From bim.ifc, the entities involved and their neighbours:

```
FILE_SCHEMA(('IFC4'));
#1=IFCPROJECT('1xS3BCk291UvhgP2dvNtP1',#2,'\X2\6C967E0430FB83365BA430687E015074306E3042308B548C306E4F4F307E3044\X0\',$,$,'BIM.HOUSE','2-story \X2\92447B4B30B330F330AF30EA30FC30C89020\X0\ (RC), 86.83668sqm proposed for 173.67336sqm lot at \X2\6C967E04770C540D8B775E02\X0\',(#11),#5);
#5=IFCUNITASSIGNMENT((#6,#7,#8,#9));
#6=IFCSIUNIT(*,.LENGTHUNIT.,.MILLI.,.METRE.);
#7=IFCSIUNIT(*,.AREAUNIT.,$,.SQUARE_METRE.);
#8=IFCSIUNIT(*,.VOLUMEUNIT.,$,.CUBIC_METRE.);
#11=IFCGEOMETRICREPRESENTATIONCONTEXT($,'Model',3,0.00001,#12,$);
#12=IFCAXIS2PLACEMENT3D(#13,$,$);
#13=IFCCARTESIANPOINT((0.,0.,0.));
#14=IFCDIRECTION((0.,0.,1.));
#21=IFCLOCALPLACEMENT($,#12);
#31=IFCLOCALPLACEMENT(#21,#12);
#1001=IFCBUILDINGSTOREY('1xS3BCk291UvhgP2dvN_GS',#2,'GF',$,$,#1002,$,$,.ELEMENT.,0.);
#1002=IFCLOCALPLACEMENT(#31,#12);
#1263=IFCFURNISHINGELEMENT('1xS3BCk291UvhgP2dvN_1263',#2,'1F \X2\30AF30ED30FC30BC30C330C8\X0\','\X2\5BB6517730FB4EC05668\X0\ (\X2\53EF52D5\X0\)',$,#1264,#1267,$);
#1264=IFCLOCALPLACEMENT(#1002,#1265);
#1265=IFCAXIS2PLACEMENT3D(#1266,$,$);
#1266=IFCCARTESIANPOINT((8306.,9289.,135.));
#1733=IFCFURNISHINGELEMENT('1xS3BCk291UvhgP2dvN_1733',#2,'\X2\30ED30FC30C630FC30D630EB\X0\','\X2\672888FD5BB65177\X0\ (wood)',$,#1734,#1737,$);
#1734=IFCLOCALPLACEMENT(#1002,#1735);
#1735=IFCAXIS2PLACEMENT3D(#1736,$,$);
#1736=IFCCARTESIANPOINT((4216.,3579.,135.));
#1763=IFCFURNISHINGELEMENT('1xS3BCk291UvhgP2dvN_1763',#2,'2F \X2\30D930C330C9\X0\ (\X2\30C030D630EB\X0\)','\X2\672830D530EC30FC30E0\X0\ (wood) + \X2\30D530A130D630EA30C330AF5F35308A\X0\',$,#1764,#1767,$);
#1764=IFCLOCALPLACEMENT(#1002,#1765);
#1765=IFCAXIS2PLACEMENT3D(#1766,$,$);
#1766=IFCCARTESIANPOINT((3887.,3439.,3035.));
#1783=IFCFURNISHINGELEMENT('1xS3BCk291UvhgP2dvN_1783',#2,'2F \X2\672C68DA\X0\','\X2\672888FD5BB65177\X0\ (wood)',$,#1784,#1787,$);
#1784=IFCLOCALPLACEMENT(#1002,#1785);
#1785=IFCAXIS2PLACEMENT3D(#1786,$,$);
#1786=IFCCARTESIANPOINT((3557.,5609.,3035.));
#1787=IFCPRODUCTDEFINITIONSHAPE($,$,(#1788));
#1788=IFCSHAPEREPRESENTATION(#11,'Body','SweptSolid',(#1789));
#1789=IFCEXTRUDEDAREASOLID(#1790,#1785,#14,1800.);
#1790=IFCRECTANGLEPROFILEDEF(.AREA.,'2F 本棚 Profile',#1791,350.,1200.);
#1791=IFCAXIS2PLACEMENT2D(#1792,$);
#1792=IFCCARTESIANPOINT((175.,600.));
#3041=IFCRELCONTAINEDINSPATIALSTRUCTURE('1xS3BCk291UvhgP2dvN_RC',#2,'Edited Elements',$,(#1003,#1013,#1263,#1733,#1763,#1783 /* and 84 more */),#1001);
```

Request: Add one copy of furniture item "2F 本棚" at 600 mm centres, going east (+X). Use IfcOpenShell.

```python
import numpy as np
import ifcopenshell
import ifcopenshell.api.geometry
import ifcopenshell.api.root
import ifcopenshell.util.element
import ifcopenshell.util.placement
import ifcopenshell.util.unit

model = ifcopenshell.open("bim.ifc")
unit_scale = ifcopenshell.util.unit.calculate_unit_scale(model)


def reuse_history(source, copy):
    """copy_class also copies each property set's owner history, people and application; keep the originals."""
    for rel in copy.IsDefinedBy:
        if rel.is_a("IfcRelDefinesByProperties") and (history := rel.RelatingPropertyDefinition.OwnerHistory):
            rel.RelatingPropertyDefinition.OwnerHistory = source.OwnerHistory
            ifcopenshell.util.element.remove_deep2(model, history)


source = model.by_guid("1xS3BCk291UvhgP2dvN_1783")
base = ifcopenshell.util.placement.get_local_placement(source.ObjectPlacement)
step = np.array([1.0, 0.0, 0.0]) * 0.6 / unit_scale

for i in range(1, 2):
    copy = ifcopenshell.api.root.copy_class(model, product=source)
    copy.Representation = ifcopenshell.util.element.copy_deep(
        model, source.Representation, exclude=["IfcGeometricRepresentationContext", "IfcRepresentationMap"]
    )
    reuse_history(source, copy)
    matrix = base.copy()
    matrix[:3, 3] += i * step
    print("added at", matrix[:3, 3].round(3) + 0.0)
    ifcopenshell.api.geometry.edit_object_placement(model, product=copy, matrix=matrix, is_si=False)

model.write("bim_updated.ifc")
```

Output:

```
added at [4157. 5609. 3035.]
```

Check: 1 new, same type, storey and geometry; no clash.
